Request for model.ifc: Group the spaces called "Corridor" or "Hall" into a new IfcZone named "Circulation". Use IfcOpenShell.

First a look at what the model holds.

```python
import ifcopenshell

model = ifcopenshell.open("model.ifc")
print(model.schema)
seen = {}
for space in model.by_type("IfcSpace"):
    seen[space.LongName] = seen.get(space.LongName, 0) + 1
for name, count in sorted(seen.items(), key=str):
    print(count, "x", name)
print("zones:", [z.Name for z in model.by_type("IfcZone")][:20])
```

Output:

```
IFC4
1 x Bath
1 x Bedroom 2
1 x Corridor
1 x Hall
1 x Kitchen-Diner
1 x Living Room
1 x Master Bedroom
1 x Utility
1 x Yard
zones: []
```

```python
import ifcopenshell
import ifcopenshell.api.group
import ifcopenshell.api.root

model = ifcopenshell.open("model.ifc")

names = {"Corridor", "Hall"}
spaces = [s for s in model.by_type("IfcSpace") if s.LongName in names]

zone = ifcopenshell.api.root.create_entity(model, ifc_class="IfcZone", name="Circulation")
ifcopenshell.api.group.assign_group(model, products=spaces, group=zone)
print(len(spaces), "spaces in", zone.Name)

model.write("model_rev.ifc")
```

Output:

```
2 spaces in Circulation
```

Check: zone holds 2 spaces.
